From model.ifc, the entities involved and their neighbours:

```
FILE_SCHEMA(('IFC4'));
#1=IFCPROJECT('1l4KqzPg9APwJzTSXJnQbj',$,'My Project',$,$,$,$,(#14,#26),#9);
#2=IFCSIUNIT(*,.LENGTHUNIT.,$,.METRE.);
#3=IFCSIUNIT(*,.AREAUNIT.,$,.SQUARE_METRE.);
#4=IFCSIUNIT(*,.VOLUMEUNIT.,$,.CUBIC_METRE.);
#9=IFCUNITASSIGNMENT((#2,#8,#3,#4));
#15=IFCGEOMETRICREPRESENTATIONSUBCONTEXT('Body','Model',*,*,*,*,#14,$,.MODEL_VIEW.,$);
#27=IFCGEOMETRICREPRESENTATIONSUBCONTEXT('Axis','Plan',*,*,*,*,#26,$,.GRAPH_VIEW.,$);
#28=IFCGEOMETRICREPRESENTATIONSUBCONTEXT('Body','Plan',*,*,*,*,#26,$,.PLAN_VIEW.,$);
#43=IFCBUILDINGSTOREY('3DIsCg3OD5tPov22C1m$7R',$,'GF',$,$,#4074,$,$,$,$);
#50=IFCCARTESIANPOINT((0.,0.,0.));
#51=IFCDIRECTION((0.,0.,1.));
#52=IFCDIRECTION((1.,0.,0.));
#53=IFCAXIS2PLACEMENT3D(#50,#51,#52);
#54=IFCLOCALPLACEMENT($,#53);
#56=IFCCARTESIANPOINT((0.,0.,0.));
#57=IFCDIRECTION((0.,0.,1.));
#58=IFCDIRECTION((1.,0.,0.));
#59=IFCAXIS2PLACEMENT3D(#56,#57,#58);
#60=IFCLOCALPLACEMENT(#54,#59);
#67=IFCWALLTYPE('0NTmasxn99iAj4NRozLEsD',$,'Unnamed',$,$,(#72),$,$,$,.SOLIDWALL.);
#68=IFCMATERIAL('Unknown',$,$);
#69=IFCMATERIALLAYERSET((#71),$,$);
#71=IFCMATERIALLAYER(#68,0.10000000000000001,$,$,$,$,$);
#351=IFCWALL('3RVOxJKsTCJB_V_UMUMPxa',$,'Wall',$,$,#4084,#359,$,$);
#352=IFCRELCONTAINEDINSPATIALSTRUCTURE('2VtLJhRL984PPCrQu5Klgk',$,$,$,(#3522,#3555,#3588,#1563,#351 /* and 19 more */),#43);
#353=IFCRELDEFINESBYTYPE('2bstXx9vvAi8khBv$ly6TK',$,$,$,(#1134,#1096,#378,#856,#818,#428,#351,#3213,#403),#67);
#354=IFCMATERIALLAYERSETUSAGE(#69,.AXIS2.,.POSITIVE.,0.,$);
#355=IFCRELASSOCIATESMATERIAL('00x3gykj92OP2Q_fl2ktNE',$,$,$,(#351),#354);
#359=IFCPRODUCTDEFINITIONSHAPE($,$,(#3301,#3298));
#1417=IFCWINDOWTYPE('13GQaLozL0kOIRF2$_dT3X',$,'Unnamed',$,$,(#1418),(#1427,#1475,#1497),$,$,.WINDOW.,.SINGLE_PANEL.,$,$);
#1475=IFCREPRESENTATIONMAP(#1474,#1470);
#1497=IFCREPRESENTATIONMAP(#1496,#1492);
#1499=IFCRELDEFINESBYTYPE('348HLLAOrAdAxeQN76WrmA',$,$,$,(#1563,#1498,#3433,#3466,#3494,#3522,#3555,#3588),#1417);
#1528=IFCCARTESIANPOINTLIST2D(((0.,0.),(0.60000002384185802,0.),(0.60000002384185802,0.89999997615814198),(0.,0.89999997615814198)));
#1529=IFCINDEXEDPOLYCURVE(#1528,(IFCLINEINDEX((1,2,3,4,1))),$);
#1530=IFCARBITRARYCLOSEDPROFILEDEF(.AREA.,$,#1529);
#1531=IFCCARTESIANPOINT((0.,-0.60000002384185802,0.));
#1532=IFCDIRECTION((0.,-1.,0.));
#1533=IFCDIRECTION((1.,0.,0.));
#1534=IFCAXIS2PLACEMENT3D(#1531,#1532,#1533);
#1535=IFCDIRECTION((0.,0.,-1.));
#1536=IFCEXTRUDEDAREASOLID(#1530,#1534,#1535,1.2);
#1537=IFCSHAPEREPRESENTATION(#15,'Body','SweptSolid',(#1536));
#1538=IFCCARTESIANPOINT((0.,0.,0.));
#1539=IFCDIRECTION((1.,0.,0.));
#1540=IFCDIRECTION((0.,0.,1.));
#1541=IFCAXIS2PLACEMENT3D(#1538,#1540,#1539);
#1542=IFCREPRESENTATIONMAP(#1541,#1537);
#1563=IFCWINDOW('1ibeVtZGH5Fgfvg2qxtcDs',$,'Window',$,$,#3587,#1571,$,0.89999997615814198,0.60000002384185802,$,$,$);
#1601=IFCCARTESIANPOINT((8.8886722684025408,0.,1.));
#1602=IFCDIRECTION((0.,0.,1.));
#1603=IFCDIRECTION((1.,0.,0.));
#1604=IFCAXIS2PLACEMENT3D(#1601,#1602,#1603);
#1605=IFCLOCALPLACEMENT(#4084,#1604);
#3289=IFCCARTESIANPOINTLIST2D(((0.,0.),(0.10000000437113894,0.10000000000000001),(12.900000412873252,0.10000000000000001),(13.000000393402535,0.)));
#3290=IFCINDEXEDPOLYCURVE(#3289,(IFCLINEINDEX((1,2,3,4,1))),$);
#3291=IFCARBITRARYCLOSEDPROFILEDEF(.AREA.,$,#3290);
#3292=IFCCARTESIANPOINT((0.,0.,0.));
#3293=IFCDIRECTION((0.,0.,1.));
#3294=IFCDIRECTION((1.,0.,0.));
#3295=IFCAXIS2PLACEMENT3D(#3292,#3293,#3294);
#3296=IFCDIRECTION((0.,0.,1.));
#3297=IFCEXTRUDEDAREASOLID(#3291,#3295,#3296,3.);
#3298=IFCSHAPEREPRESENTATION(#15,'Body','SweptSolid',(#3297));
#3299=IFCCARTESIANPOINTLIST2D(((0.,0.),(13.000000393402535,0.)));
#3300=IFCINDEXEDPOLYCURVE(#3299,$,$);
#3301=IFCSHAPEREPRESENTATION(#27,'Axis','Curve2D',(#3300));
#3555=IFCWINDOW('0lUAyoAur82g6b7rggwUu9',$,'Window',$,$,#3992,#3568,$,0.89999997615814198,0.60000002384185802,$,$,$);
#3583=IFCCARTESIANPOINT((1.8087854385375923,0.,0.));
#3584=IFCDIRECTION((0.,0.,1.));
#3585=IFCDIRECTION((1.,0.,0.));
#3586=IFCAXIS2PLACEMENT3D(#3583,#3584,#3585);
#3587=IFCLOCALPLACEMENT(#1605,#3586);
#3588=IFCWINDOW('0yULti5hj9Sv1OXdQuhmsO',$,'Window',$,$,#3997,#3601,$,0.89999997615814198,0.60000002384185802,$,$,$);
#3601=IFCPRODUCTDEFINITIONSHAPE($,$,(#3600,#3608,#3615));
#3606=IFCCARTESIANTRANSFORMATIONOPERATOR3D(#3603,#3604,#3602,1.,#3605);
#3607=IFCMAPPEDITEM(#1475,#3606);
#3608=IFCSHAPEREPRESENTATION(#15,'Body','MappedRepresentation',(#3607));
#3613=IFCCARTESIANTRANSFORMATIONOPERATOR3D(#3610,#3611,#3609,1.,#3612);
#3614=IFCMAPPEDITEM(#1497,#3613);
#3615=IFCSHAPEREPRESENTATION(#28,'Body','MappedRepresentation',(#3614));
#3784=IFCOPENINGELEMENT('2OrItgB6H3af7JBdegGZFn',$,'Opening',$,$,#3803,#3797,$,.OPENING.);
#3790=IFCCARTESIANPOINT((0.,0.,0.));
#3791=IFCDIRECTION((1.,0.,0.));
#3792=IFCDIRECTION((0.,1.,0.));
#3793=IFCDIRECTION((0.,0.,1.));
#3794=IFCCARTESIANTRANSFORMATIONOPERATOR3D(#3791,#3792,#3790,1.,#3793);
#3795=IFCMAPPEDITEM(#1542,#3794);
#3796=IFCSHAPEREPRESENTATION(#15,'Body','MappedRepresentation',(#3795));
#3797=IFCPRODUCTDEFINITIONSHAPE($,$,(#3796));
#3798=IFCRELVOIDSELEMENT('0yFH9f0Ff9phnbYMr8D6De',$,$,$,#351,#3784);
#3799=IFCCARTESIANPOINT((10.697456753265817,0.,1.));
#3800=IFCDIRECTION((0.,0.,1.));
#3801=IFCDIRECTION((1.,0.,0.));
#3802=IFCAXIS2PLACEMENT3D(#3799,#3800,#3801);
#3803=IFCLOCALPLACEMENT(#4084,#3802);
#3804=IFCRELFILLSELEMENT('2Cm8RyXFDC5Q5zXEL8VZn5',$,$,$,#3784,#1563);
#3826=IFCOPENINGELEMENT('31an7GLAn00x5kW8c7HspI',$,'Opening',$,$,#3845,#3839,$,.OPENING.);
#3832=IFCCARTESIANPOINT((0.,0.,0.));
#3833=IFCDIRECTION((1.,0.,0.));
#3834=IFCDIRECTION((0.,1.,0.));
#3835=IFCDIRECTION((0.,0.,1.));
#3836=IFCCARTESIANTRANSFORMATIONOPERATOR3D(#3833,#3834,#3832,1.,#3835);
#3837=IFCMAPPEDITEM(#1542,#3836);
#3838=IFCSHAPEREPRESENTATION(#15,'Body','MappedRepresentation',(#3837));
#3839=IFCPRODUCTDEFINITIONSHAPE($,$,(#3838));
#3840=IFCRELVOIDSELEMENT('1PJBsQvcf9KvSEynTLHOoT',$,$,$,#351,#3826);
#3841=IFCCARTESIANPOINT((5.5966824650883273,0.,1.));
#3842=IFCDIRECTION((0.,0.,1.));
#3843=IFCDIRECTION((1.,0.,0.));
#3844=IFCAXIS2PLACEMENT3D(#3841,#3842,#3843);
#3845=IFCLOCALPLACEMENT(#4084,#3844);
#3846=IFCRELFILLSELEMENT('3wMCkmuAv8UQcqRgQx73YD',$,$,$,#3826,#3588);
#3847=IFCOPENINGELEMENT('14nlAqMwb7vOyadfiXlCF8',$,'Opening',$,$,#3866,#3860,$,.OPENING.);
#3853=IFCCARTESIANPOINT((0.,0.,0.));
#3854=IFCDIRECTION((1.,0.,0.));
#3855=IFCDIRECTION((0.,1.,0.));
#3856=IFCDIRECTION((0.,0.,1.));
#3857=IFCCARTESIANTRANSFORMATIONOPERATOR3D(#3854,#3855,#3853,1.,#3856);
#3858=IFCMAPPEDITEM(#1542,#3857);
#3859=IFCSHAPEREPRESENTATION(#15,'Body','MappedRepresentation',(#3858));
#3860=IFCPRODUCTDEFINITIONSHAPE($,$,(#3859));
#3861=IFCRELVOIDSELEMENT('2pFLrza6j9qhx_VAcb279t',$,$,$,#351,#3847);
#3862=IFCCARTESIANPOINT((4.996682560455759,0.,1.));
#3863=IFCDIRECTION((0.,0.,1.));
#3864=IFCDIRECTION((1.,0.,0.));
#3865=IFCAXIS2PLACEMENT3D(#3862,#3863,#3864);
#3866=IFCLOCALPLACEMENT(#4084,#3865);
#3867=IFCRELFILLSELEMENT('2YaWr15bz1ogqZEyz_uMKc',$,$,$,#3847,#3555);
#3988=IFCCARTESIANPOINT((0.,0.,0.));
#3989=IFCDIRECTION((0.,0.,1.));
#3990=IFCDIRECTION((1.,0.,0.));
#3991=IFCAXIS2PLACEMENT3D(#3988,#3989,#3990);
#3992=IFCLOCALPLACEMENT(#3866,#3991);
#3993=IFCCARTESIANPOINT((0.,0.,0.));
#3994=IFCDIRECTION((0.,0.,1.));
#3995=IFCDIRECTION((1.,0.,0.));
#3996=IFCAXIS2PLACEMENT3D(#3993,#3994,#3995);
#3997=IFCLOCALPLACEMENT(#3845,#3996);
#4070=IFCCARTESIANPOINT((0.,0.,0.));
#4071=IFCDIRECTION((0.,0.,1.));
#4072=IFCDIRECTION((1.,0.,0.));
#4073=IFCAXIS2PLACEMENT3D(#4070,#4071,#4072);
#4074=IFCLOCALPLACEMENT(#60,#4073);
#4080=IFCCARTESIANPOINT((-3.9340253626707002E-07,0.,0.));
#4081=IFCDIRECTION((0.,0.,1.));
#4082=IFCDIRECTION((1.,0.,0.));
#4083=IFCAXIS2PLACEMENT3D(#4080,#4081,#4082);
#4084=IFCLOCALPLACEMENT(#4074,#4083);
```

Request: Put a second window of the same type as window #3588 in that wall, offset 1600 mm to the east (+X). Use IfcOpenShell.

```python
import ifcopenshell
import ifcopenshell.api.feature
import ifcopenshell.api.geometry
import ifcopenshell.api.root
import ifcopenshell.geom
import ifcopenshell.util.element
import ifcopenshell.util.placement
import ifcopenshell.util.shape
import ifcopenshell.util.unit

model = ifcopenshell.open("model.ifc")
unit_scale = ifcopenshell.util.unit.calculate_unit_scale(model)
settings = ifcopenshell.geom.settings()


def volume(element):
    """Net volume in cubic metres, openings subtracted."""
    shape = ifcopenshell.geom.create_shape(settings, element)
    return ifcopenshell.util.shape.get_volume(shape.geometry)


window = model.by_guid("0yULti5hj9Sv1OXdQuhmsO")
opening = window.FillsVoids[0].RelatingOpeningElement
wall = opening.VoidsElements[0].RelatingBuildingElement
before = volume(wall)
shift = ifcopenshell.util.placement.get_local_placement(wall.ObjectPlacement)[:3, 0] * 1.6 / unit_scale

# copy_class copies the void relationship, type, container and properties, but no geometry.
new_opening = ifcopenshell.api.root.copy_class(model, product=opening)
new_opening.Representation = ifcopenshell.util.element.copy_deep(
    model, opening.Representation, exclude=["IfcGeometricRepresentationContext", "IfcRepresentationMap"]
)
new_window = ifcopenshell.api.root.copy_class(model, product=window)
new_window.Representation = ifcopenshell.util.element.copy_deep(
    model, window.Representation, exclude=["IfcGeometricRepresentationContext", "IfcRepresentationMap"]
)
ifcopenshell.api.feature.add_filling(model, opening=new_opening, element=new_window)

for old, new in ((opening, new_opening), (window, new_window)):
    matrix = ifcopenshell.util.placement.get_local_placement(old.ObjectPlacement)
    matrix[:3, 3] += shift
    ifcopenshell.api.geometry.edit_object_placement(model, product=new, matrix=matrix, is_si=False)

after = volume(wall)

print(f"wall volume {before:.3f} -> {after:.3f} m3")

model.write("model-out.ifc")
```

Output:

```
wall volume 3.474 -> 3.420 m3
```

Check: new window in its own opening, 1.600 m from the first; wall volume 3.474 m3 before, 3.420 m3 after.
